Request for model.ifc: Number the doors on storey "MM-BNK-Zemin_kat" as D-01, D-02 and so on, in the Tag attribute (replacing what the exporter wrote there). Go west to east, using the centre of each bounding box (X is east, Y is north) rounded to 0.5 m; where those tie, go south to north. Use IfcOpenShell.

First a look at what the model holds.

```python
import ifcopenshell
import ifcopenshell.util.element
import ifcopenshell.util.placement

model = ifcopenshell.open("model.ifc")
print(model.schema)
storey = next(s for s in model.by_type("IfcBuildingStorey") if s.Name == "MM-BNK-Zemin_kat")
doors = [e for e in ifcopenshell.util.element.get_decomposition(storey) if e.is_a("IfcDoor")]
for e in sorted(doors, key=lambda e: e.id()):
    origin = ifcopenshell.util.placement.get_local_placement(e.ObjectPlacement)[:3, 3]
    print(e.id(), e.Tag, e.Name, origin.round(2) + 0.0, sep=" | ")
```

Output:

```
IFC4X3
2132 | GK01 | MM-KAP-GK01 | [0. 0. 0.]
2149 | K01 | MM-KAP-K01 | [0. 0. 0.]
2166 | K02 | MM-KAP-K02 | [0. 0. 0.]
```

```python
import ifcopenshell
import ifcopenshell.geom
import ifcopenshell.util.element
import ifcopenshell.util.shape

model = ifcopenshell.open("model.ifc")
settings = ifcopenshell.geom.settings()
settings.set("use-world-coords", True)


def centre(element):
    shape = ifcopenshell.geom.create_shape(settings, element)
    return ifcopenshell.util.shape.get_bbox_centroid(shape.geometry)


storey = next(s for s in model.by_type("IfcBuildingStorey") if s.Name == "MM-BNK-Zemin_kat")
doors = [e for e in ifcopenshell.util.element.get_decomposition(storey) if e.is_a("IfcDoor")]

# Insertion points can sit at a corner or the storey origin, so sort by the geometry (in metres).
centres = {e: centre(e) for e in doors}
doors.sort(key=lambda e: (round(centres[e][0] / 0.5), centres[e][1]))

for i, e in enumerate(doors, start=1):
    number = f"D-{i:02d}"
    e.Tag = number
    print(e.id(), number)

model.write("model_edited.ifc")
```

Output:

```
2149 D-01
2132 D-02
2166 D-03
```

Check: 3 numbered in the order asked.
